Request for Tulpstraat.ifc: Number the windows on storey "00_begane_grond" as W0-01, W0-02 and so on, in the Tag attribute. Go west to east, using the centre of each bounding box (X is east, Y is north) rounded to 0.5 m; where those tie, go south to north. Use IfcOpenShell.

First a look at what the model holds.

```python
import ifcopenshell
import ifcopenshell.util.element
import ifcopenshell.util.placement

model = ifcopenshell.open("Tulpstraat.ifc")
print(model.schema)
storey = next(s for s in model.by_type("IfcBuildingStorey") if s.Name == "00_begane_grond")
windows = [e for e in ifcopenshell.util.element.get_decomposition(storey) if e.is_a("IfcWindow")]
for e in sorted(windows, key=lambda e: e.id()):
    origin = ifcopenshell.util.placement.get_local_placement(e.ObjectPlacement)[:3, 3]
    print(e.id(), e.Tag, e.Name, origin.round(2) + 0.0, sep=" | ")
```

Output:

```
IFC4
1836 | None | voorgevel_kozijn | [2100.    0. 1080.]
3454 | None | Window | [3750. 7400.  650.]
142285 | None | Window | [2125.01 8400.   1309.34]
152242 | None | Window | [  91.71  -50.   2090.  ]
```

```python
import ifcopenshell
import ifcopenshell.geom
import ifcopenshell.util.element
import ifcopenshell.util.shape

model = ifcopenshell.open("Tulpstraat.ifc")
settings = ifcopenshell.geom.settings()
settings.set("use-world-coords", True)


def centre(element):
    shape = ifcopenshell.geom.create_shape(settings, element)
    return ifcopenshell.util.shape.get_bbox_centroid(shape.geometry)


storey = next(s for s in model.by_type("IfcBuildingStorey") if s.Name == "00_begane_grond")
windows = [e for e in ifcopenshell.util.element.get_decomposition(storey) if e.is_a("IfcWindow")]

# Insertion points can sit at a corner or the storey origin, so sort by the geometry (in metres).
centres = {e: centre(e) for e in windows}
windows.sort(key=lambda e: (round(centres[e][0] / 0.5), centres[e][1]))

for i, e in enumerate(windows, start=1):
    number = f"W0-{i:02d}"
    e.Tag = number
    print(e.id(), number)

model.write("Tulpstraat_v2.ifc")
```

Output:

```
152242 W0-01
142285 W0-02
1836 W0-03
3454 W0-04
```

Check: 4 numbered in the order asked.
